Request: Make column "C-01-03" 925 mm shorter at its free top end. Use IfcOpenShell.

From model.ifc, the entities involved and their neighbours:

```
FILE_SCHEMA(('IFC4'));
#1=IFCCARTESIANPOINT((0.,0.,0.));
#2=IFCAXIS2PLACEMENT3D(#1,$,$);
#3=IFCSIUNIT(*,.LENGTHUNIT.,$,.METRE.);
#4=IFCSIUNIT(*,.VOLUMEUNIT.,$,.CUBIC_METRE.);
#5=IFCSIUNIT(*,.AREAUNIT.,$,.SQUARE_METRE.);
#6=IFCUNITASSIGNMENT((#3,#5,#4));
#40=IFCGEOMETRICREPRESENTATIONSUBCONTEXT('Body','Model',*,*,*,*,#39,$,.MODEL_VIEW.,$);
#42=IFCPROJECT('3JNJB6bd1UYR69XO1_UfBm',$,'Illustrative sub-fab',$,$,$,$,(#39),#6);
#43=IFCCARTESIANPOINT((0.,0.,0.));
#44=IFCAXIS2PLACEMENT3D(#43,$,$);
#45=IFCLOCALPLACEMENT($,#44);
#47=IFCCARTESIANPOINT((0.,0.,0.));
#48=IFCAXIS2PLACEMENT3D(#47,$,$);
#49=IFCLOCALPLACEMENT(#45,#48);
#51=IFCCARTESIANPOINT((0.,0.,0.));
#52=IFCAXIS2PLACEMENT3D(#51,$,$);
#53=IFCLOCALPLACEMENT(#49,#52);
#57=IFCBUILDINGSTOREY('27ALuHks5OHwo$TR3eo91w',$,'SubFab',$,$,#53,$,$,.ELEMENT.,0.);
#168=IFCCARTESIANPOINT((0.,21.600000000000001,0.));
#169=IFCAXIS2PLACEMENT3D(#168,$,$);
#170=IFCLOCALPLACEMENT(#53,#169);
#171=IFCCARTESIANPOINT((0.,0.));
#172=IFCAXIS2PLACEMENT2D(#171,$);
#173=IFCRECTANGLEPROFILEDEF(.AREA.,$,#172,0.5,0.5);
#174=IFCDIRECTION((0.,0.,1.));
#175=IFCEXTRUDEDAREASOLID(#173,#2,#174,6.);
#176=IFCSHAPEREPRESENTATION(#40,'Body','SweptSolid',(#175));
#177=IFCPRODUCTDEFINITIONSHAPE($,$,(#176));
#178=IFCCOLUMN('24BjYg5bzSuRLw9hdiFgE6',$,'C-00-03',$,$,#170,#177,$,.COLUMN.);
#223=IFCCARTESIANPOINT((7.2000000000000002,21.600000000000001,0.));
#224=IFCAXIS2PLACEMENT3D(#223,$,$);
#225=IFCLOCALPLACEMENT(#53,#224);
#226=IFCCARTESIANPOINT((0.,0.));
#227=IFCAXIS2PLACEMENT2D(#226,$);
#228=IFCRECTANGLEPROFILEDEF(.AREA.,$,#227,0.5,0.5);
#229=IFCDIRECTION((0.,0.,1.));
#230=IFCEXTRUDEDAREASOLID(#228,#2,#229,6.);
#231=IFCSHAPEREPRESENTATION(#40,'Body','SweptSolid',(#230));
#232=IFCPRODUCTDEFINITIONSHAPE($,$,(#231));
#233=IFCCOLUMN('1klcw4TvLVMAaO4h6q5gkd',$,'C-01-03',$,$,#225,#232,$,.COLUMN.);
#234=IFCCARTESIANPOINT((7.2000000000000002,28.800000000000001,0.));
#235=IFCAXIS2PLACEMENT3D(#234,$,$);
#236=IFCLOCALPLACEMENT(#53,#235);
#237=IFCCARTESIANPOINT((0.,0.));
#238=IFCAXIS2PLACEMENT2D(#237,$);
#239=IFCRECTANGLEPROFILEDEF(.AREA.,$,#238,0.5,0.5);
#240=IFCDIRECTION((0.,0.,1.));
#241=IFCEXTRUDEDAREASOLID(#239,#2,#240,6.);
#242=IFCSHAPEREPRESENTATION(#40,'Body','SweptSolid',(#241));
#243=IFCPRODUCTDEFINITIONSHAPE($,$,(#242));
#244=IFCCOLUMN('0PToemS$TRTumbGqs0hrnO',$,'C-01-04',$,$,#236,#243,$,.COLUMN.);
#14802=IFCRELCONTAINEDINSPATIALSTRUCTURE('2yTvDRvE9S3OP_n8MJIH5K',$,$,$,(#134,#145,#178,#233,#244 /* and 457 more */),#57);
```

```python
import ifcopenshell
import ifcopenshell.util.representation

model = ifcopenshell.open("model.ifc")

member = model.by_guid("1klcw4TvLVMAaO4h6q5gkd")
change = -0.925

# The extrusion runs towards the end named, so only its depth changes.
body = ifcopenshell.util.representation.get_representation(member, "Model", "Body")
solid = body.Items[0]
old_length = solid.Depth
solid.Depth += change

print(f"length {old_length:g} -> {solid.Depth:g}")

model.write("model_v2.ifc")
```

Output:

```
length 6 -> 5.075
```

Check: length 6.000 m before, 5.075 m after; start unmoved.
